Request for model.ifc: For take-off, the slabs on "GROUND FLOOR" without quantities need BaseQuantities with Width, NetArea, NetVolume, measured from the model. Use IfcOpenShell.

First a look at what the model holds.

```python
import ifcopenshell
import ifcopenshell.util.element
import ifcopenshell.util.unit

model = ifcopenshell.open("model.ifc")
print(model.schema)
for unit_type in ("LENGTHUNIT", "AREAUNIT", "VOLUMEUNIT"):
    print(unit_type, ifcopenshell.util.unit.calculate_unit_scale(model, unit_type))
storey = next(s for s in model.by_type("IfcBuildingStorey") if s.Name == "GROUND FLOOR")
slabs = [e for e in ifcopenshell.util.element.get_decomposition(storey) if e.is_a("IfcSlab")]
for e in sorted(slabs, key=lambda e: e.id()):
    print(e.id(), e.is_a(), e.Name, list(ifcopenshell.util.element.get_psets(e, qtos_only=True)), sep=" | ")
```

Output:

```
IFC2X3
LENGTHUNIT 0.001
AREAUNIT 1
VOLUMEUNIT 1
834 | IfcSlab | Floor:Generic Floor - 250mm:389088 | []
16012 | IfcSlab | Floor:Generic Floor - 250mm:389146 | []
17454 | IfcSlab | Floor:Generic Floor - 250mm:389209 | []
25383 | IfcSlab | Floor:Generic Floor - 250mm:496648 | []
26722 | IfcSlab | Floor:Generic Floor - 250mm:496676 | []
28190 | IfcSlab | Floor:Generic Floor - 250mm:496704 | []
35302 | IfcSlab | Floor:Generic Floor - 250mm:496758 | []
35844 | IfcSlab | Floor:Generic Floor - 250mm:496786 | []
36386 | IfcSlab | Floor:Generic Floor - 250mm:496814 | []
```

```python
import ifcopenshell
import ifcopenshell.api.pset
import ifcopenshell.geom
import ifcopenshell.util.element
import ifcopenshell.util.shape
import ifcopenshell.util.unit

model = ifcopenshell.open("model.ifc")
unit_scale = ifcopenshell.util.unit.calculate_unit_scale(model)
area_scale = ifcopenshell.util.unit.calculate_unit_scale(model, "AREAUNIT")
volume_scale = ifcopenshell.util.unit.calculate_unit_scale(model, "VOLUMEUNIT")
settings = ifcopenshell.geom.settings()

storey = next(s for s in model.by_type("IfcBuildingStorey") if s.Name == "GROUND FLOOR")
slabs = [e for e in ifcopenshell.util.element.get_decomposition(storey) if e.is_a("IfcSlab")]

for e in sorted(slabs, key=lambda e: e.id()):
    if ifcopenshell.util.element.get_psets(e, qtos_only=True, should_inherit=False):
        continue
    # Geometry comes back in metres, in the element's own axes.
    shape = ifcopenshell.geom.create_shape(settings, e)
    values = {
        "Width": ifcopenshell.util.shape.get_z(shape.geometry) / unit_scale,
        "NetArea": ifcopenshell.util.shape.get_footprint_area(shape.geometry) / area_scale,
        "NetVolume": ifcopenshell.util.shape.get_volume(shape.geometry) / volume_scale,
    }
    qto = ifcopenshell.api.pset.add_qto(model, product=e, name="BaseQuantities")
    ifcopenshell.api.pset.edit_qto(model, qto=qto, properties=values)
    print(e.id(), {k: round(v, 3) for k, v in values.items()})

model.write("model_updated.ifc")
```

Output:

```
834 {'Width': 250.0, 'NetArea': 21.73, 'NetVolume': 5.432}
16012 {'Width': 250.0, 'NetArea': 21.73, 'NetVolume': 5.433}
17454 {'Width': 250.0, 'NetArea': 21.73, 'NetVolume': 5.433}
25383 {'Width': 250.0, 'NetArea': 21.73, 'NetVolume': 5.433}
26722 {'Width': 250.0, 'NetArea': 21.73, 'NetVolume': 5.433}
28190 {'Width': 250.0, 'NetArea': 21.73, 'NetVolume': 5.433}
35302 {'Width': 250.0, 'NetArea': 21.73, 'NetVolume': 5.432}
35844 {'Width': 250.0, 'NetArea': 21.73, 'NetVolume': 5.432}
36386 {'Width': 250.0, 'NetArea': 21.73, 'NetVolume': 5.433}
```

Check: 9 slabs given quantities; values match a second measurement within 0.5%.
